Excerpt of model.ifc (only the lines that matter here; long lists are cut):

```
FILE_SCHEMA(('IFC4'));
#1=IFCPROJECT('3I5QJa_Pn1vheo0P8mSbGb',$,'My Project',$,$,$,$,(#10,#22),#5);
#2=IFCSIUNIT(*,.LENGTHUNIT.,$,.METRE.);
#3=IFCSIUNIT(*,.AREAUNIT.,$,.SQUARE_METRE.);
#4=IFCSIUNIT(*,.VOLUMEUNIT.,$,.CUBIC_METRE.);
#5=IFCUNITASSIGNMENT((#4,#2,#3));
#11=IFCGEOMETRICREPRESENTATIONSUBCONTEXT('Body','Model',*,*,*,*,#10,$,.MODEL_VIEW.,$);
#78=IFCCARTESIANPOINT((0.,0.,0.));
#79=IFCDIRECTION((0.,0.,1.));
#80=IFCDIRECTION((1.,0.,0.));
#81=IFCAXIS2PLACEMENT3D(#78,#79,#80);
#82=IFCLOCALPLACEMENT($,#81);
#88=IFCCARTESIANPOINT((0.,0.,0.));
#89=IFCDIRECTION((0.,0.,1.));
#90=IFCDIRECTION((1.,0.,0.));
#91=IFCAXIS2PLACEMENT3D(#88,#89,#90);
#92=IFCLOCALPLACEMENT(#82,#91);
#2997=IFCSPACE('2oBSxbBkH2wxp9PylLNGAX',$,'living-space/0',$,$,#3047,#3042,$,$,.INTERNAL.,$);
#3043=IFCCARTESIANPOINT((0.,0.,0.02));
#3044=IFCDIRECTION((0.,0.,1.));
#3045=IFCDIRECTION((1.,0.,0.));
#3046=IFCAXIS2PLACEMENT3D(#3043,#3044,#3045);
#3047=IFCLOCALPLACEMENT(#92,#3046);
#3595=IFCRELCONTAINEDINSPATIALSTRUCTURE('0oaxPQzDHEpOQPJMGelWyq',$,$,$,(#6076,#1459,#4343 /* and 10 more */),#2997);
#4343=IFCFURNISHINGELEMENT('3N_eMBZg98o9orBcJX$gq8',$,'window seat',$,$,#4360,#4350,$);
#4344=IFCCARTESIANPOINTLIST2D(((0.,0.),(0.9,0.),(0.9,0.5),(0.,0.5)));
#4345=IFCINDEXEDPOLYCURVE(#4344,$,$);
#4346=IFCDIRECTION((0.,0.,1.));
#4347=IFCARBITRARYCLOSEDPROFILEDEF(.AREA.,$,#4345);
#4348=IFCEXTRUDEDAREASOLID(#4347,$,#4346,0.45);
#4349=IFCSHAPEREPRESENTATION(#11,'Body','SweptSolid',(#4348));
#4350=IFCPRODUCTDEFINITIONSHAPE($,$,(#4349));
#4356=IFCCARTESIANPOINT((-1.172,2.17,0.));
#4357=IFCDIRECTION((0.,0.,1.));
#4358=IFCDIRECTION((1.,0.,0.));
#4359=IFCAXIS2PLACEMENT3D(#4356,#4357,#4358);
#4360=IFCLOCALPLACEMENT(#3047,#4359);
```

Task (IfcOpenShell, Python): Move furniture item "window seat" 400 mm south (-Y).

```python
import ifcopenshell
import ifcopenshell.api.geometry
import ifcopenshell.util.placement

model = ifcopenshell.open("model.ifc")

item = model.by_guid("3N_eMBZg98o9orBcJX$gq8")
matrix = ifcopenshell.util.placement.get_local_placement(item.ObjectPlacement)
matrix[1, 3] -= 0.4
ifcopenshell.api.geometry.edit_object_placement(model, product=item, matrix=matrix, is_si=False)

print(ifcopenshell.util.placement.get_local_placement(item.ObjectPlacement).round(3) + 0.0)

model.write("model_edited.ifc")
```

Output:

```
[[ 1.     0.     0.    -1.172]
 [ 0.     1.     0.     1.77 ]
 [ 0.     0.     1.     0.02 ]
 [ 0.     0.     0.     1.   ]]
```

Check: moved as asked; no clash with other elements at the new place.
